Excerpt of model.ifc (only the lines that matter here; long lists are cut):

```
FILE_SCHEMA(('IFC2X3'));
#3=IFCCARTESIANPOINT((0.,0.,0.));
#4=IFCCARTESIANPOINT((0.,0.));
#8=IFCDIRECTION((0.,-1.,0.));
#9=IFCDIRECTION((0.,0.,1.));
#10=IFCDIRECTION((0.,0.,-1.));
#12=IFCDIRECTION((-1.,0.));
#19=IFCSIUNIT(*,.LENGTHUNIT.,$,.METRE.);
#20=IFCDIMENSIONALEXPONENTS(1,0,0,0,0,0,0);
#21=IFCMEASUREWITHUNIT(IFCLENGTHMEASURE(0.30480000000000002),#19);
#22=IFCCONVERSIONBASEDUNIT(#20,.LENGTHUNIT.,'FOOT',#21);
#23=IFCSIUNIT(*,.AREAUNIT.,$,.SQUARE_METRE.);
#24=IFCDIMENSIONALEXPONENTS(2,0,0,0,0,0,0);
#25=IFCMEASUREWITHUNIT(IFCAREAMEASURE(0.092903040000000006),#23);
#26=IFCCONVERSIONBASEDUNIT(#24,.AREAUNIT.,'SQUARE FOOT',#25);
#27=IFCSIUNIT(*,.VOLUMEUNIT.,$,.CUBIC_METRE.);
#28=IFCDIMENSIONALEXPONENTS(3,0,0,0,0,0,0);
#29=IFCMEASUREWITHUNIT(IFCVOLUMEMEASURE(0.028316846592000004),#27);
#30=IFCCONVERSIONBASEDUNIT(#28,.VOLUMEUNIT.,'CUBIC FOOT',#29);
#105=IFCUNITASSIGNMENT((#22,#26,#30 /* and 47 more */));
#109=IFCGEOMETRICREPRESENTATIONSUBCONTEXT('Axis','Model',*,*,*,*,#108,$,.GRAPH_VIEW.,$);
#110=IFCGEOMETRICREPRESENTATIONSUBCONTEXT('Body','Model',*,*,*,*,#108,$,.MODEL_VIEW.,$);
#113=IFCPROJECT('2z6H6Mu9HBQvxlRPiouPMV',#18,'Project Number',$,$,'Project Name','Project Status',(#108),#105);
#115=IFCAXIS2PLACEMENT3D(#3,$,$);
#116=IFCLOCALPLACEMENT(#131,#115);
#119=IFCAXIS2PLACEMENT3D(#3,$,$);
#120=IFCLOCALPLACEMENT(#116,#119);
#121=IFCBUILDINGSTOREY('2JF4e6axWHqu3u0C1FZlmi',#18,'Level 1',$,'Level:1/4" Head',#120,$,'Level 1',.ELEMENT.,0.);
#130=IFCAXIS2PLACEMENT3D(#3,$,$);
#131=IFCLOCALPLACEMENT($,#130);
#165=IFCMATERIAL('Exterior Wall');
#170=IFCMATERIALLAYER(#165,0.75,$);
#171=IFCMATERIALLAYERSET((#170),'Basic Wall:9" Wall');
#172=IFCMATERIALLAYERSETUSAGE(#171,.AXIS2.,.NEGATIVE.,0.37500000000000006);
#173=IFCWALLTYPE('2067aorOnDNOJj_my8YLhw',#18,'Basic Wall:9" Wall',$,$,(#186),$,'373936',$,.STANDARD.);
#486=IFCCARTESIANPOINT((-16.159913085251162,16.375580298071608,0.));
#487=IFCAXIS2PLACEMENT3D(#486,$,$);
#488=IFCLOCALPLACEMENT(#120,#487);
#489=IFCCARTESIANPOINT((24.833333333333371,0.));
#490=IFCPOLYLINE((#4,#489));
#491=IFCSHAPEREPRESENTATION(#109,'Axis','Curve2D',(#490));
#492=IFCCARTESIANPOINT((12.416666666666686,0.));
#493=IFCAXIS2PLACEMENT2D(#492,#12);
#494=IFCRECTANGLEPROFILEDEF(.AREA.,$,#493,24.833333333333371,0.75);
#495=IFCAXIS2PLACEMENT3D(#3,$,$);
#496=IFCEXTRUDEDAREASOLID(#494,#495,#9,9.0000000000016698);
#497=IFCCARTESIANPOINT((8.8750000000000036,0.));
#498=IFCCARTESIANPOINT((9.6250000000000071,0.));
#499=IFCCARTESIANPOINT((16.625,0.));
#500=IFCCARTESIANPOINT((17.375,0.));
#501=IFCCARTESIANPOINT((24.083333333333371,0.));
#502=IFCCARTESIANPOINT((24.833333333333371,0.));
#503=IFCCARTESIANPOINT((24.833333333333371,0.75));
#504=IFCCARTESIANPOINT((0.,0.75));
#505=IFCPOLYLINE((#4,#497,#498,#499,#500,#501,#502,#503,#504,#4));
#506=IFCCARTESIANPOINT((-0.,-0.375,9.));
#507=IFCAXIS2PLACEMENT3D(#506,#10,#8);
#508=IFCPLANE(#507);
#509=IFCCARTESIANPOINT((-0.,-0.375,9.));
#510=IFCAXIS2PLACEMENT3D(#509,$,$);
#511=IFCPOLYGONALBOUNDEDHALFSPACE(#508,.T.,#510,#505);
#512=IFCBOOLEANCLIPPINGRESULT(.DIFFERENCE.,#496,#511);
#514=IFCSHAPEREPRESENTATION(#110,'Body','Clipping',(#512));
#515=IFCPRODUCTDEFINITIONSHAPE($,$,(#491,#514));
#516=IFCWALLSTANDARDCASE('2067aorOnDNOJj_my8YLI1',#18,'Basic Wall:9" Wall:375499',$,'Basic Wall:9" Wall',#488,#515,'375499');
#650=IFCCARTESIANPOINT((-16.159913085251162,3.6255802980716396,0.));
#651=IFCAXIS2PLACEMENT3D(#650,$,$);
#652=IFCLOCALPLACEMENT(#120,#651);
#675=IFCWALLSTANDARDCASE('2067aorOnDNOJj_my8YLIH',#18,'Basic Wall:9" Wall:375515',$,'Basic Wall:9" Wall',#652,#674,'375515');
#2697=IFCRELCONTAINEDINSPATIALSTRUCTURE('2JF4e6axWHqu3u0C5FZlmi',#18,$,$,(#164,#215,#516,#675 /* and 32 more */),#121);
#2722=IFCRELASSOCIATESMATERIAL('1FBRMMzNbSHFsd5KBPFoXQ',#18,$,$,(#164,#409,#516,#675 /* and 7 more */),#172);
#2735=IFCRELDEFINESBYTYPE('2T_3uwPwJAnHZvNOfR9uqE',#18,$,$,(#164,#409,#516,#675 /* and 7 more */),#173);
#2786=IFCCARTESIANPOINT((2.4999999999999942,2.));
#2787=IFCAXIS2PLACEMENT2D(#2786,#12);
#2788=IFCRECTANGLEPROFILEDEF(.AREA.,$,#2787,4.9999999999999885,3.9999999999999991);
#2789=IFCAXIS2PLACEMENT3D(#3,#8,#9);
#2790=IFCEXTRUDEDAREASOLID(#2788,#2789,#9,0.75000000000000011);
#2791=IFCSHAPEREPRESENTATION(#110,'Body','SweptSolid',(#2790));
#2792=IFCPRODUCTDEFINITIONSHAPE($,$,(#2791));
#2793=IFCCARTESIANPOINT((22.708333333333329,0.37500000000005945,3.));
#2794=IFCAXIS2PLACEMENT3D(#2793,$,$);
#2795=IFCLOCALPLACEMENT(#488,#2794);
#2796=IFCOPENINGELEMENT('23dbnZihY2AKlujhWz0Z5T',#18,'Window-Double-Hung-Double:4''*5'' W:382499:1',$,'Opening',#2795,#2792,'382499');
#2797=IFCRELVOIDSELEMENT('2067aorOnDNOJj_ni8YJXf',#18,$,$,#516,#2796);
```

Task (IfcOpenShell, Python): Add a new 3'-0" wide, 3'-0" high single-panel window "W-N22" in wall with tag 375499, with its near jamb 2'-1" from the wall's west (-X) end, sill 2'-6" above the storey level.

```python
import numpy as np
import ifcopenshell
import ifcopenshell.api.feature
import ifcopenshell.api.geometry
import ifcopenshell.api.root
import ifcopenshell.api.spatial
import ifcopenshell.api.type
import ifcopenshell.geom
import ifcopenshell.util.element
import ifcopenshell.util.placement
import ifcopenshell.util.representation
import ifcopenshell.util.shape
import ifcopenshell.util.unit

model = ifcopenshell.open("model.ifc")
unit_scale = ifcopenshell.util.unit.calculate_unit_scale(model)
settings = ifcopenshell.geom.settings()


def volume(element):
    """Net volume in cubic metres, openings subtracted."""
    shape = ifcopenshell.geom.create_shape(settings, element)
    return ifcopenshell.util.shape.get_volume(shape.geometry)


wall = model.by_guid("2067aorOnDNOJj_my8YLI1")
storey = ifcopenshell.util.element.get_container(wall, ifc_class="IfcBuildingStorey")
context = ifcopenshell.util.representation.get_context(model, "Model", "Body", "MODEL_VIEW")
before = volume(wall)

width, height, from_end, sill = 0.9144, 0.9144, 0.635, 0.762  # metres

# The wall runs along its own X axis, and the end named is its -X end.
wall_shape = ifcopenshell.geom.create_shape(settings, wall)
x, y, z = ifcopenshell.util.shape.get_vertices(wall_shape.geometry).T
start = x.min() + from_end
face, thickness = float(y.min()), float(y.max() - y.min())
wall_matrix = ifcopenshell.util.placement.get_local_placement(wall.ObjectPlacement)
level = ifcopenshell.util.placement.get_local_placement(storey.ObjectPlacement)[2, 3]


def in_wall(x, y):
    """Placement at x, y metres in the wall's axes, at sill height."""
    matrix = wall_matrix.copy()
    matrix[:, 3] = wall_matrix @ np.array([x / unit_scale, y / unit_scale, 0.0, 1.0])
    matrix[2, 3] = level + sill / unit_scale
    return matrix


# Opening: a box that overshoots both wall faces by 50 mm.
opening = ifcopenshell.api.root.create_entity(model, ifc_class="IfcOpeningElement")
box = ifcopenshell.api.geometry.add_wall_representation(
    model, context=context, length=width, height=height, thickness=thickness + 0.1
)
ifcopenshell.api.geometry.assign_representation(model, product=opening, representation=box)
ifcopenshell.api.geometry.edit_object_placement(model, product=opening, matrix=in_wall(start, face - 0.05), is_si=False)
ifcopenshell.api.feature.add_feature(model, feature=opening, element=wall)

window = ifcopenshell.api.root.create_entity(model, ifc_class="IfcWindow", name="W-N22")
window.OverallWidth, window.OverallHeight = width / unit_scale, height / unit_scale
body = ifcopenshell.api.geometry.add_window_representation(
    model,
    context=context,
    overall_width=window.OverallWidth,
    overall_height=window.OverallHeight,
    partition_type="SINGLE_PANEL",
)
ifcopenshell.api.geometry.assign_representation(model, product=window, representation=body)
ifcopenshell.api.spatial.assign_container(model, products=[window], relating_structure=storey)
fills = ifcopenshell.api.feature.add_filling(model, opening=opening, element=window)
fills.OwnerHistory = window.OwnerHistory  # required in IFC2X3

# IFC2X3 keeps the operation on the window style.
style = ifcopenshell.api.root.create_entity(model, ifc_class="IfcWindowStyle", name="W-N22")
style.OperationType, style.ConstructionType = "SINGLE_PANEL", "NOTDEFINED"
style.ParameterTakesPrecedence = style.Sizeable = False
ifcopenshell.api.type.assign_type(model, related_objects=[window], relating_type=style)

# Centre the window in the wall's thickness.
ifcopenshell.api.geometry.edit_object_placement(model, product=window, matrix=in_wall(start, face), is_si=False)
window_shape = ifcopenshell.geom.create_shape(settings, window)
depth = ifcopenshell.util.shape.get_vertices(window_shape.geometry)[:, 1]
offset = face + thickness / 2 - (depth.min() + depth.max()) / 2
ifcopenshell.api.geometry.edit_object_placement(model, product=window, matrix=in_wall(start, offset), is_si=False)

after = volume(wall)

print(f"wall volume {before:.3f} -> {after:.3f} m3")

model.write("model_updated.ifc")
```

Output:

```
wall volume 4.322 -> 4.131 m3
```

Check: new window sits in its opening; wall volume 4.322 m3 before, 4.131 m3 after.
